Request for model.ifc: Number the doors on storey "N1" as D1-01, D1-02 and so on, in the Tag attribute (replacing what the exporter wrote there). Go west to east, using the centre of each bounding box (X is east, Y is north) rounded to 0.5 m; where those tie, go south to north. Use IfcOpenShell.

First a look at what the model holds.

```python
import ifcopenshell
import ifcopenshell.util.element
import ifcopenshell.util.placement

model = ifcopenshell.open("model.ifc")
print(model.schema)
storey = next(s for s in model.by_type("IfcBuildingStorey") if s.Name == "N1")
doors = [e for e in ifcopenshell.util.element.get_decomposition(storey) if e.is_a("IfcDoor")]
for e in sorted(doors, key=lambda e: e.id()):
    origin = ifcopenshell.util.placement.get_local_placement(e.ObjectPlacement)[:3, 3]
    print(e.id(), e.Tag, e.Name, origin.round(2) + 0.0, sep=" | ")
```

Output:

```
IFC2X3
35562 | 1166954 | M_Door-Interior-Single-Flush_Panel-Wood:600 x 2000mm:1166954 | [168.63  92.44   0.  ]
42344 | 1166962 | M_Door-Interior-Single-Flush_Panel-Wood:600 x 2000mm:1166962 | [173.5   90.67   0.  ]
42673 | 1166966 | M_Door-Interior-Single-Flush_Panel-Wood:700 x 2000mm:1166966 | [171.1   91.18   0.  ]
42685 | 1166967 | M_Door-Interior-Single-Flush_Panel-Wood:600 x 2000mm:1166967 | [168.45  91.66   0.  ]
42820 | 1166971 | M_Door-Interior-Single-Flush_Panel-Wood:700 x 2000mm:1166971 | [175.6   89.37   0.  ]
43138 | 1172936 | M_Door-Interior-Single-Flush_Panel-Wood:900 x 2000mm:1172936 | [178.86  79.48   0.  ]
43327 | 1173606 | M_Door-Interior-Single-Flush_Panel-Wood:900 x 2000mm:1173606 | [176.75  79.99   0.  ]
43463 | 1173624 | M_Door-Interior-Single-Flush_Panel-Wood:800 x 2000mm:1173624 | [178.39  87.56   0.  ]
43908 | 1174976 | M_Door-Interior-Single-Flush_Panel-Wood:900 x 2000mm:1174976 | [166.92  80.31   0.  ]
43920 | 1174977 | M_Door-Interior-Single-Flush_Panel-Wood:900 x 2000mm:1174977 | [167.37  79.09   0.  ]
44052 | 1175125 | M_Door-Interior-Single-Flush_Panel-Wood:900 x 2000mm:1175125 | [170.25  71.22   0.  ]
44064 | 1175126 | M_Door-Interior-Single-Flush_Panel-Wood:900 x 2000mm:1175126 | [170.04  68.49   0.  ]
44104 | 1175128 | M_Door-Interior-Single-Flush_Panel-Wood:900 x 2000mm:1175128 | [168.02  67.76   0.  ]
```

```python
import ifcopenshell
import ifcopenshell.geom
import ifcopenshell.util.element
import ifcopenshell.util.shape

model = ifcopenshell.open("model.ifc")
settings = ifcopenshell.geom.settings()
settings.set("use-world-coords", True)


def centre(element):
    shape = ifcopenshell.geom.create_shape(settings, element)
    return ifcopenshell.util.shape.get_bbox_centroid(shape.geometry)


storey = next(s for s in model.by_type("IfcBuildingStorey") if s.Name == "N1")
doors = [e for e in ifcopenshell.util.element.get_decomposition(storey) if e.is_a("IfcDoor")]

# Insertion points can sit at a corner or the storey origin, so sort by the geometry (in metres).
centres = {e: centre(e) for e in doors}
doors.sort(key=lambda e: (round(centres[e][0] / 0.5), centres[e][1]))

for i, e in enumerate(doors, start=1):
    number = f"D1-{i:02d}"
    e.Tag = number
    print(e.id(), number)

model.write("model_updated.ifc")
```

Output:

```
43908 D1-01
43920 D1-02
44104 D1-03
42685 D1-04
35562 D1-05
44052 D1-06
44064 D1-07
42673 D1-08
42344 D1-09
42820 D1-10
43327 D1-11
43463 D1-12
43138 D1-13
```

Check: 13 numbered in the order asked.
